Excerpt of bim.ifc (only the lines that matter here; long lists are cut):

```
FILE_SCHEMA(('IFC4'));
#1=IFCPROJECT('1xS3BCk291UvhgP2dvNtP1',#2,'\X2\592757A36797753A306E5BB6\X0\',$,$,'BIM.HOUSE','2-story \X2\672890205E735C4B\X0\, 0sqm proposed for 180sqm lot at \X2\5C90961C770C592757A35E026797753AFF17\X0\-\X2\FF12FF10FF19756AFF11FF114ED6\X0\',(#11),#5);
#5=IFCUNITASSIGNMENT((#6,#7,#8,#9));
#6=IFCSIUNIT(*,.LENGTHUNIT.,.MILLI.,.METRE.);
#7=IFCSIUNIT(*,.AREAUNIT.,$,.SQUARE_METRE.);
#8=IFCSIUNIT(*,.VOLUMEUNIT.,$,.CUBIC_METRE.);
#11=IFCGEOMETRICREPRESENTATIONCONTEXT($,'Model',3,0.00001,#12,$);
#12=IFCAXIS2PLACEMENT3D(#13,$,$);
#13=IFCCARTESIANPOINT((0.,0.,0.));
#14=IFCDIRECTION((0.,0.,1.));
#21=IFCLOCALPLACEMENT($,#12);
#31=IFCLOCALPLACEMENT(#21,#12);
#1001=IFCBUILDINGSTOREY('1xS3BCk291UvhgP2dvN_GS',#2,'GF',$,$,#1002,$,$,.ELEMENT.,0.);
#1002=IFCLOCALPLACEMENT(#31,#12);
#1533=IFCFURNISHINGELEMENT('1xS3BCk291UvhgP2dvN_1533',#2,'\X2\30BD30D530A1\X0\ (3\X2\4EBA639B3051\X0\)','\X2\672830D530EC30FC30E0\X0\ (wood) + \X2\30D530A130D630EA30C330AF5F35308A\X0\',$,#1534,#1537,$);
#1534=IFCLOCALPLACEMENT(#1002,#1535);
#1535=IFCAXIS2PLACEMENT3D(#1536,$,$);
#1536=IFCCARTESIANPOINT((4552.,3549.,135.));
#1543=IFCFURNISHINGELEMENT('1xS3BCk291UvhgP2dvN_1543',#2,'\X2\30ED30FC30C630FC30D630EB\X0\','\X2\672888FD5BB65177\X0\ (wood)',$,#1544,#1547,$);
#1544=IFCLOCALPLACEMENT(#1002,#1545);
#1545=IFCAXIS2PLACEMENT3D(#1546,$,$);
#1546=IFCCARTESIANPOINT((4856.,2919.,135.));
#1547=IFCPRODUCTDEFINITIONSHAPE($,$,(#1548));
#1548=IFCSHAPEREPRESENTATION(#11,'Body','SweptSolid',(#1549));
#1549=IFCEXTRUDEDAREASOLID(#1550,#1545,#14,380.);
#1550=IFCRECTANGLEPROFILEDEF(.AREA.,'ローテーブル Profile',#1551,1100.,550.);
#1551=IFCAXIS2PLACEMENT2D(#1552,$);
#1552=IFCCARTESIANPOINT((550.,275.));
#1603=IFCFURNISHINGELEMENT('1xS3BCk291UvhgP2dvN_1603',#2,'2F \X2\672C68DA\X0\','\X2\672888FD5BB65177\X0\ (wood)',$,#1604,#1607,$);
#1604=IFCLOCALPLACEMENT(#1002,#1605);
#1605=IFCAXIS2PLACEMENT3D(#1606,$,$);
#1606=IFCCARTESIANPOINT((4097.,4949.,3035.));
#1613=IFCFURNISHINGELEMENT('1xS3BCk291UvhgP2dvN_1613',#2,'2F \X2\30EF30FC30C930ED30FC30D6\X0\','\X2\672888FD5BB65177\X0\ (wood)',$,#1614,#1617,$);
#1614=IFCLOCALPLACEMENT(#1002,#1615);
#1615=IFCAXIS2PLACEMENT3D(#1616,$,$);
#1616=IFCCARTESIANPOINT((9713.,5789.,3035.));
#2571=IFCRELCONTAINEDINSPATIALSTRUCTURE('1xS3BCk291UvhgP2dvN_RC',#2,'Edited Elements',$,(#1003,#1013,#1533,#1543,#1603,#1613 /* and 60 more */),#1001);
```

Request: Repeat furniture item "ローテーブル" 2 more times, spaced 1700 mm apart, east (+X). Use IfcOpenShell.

```python
import numpy as np
import ifcopenshell
import ifcopenshell.api.geometry
import ifcopenshell.api.root
import ifcopenshell.util.element
import ifcopenshell.util.placement

model = ifcopenshell.open("bim.ifc")


def reuse_history(source, copy):
    """copy_class also copies each property set's owner history, people and application; keep the originals."""
    for rel in copy.IsDefinedBy:
        if rel.is_a("IfcRelDefinesByProperties") and (history := rel.RelatingPropertyDefinition.OwnerHistory):
            rel.RelatingPropertyDefinition.OwnerHistory = source.OwnerHistory
            ifcopenshell.util.element.remove_deep2(model, history)


source = model.by_guid("1xS3BCk291UvhgP2dvN_1543")
base = ifcopenshell.util.placement.get_local_placement(source.ObjectPlacement)
step = np.array([1.0, 0.0, 0.0]) * 1700.0

for i in range(1, 3):
    copy = ifcopenshell.api.root.copy_class(model, product=source)
    copy.Representation = ifcopenshell.util.element.copy_deep(
        model, source.Representation, exclude=["IfcGeometricRepresentationContext", "IfcRepresentationMap"]
    )
    reuse_history(source, copy)
    matrix = base.copy()
    matrix[:3, 3] += i * step
    print("added at", matrix[:3, 3].round(3) + 0.0)
    ifcopenshell.api.geometry.edit_object_placement(model, product=copy, matrix=matrix, is_si=False)

model.write("bim_v2.ifc")
```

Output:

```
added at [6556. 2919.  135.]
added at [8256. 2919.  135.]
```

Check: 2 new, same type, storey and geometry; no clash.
